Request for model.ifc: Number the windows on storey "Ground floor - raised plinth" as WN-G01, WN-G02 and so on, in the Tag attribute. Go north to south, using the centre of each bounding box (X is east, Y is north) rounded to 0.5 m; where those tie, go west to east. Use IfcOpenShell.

First a look at what the model holds.

```python
import ifcopenshell
import ifcopenshell.util.element
import ifcopenshell.util.placement

model = ifcopenshell.open("model.ifc")
print(model.schema)
storey = next(s for s in model.by_type("IfcBuildingStorey") if s.Name == "Ground floor - raised plinth")
windows = [e for e in ifcopenshell.util.element.get_decomposition(storey) if e.is_a("IfcWindow")]
for e in sorted(windows, key=lambda e: e.id()):
    origin = ifcopenshell.util.placement.get_local_placement(e.ObjectPlacement)[:3, 3]
    print(e.id(), e.Tag, e.Name, origin.round(2) + 0.0, sep=" | ")
```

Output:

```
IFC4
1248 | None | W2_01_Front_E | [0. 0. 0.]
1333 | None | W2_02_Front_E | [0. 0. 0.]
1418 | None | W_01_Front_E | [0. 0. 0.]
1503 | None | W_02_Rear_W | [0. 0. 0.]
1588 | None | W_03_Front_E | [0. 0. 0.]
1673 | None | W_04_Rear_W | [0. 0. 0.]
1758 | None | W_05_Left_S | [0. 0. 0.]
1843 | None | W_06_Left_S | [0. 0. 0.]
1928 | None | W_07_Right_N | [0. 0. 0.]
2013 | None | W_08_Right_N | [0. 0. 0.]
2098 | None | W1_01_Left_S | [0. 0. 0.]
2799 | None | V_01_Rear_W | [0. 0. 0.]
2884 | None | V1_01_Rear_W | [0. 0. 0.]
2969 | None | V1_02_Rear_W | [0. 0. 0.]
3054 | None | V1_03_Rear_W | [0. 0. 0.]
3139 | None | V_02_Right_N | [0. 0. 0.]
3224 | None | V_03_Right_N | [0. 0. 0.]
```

```python
import ifcopenshell
import ifcopenshell.geom
import ifcopenshell.util.element
import ifcopenshell.util.shape

model = ifcopenshell.open("model.ifc")
settings = ifcopenshell.geom.settings()
settings.set("use-world-coords", True)


def centre(element):
    shape = ifcopenshell.geom.create_shape(settings, element)
    return ifcopenshell.util.shape.get_bbox_centroid(shape.geometry)


storey = next(s for s in model.by_type("IfcBuildingStorey") if s.Name == "Ground floor - raised plinth")
windows = [e for e in ifcopenshell.util.element.get_decomposition(storey) if e.is_a("IfcWindow")]

# Insertion points can sit at a corner or the storey origin, so sort by the geometry (in metres).
centres = {e: centre(e) for e in windows}
windows.sort(key=lambda e: (-round(centres[e][1] / 0.5), centres[e][0]))

for i, e in enumerate(windows, start=1):
    number = f"WN-G{i:02d}"
    e.Tag = number
    print(e.id(), number)

model.write("model_edited.ifc")
```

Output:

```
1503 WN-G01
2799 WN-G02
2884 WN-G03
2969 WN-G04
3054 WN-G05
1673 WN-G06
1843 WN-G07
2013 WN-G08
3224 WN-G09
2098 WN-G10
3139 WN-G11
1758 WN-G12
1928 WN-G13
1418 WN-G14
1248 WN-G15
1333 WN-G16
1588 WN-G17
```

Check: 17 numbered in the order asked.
